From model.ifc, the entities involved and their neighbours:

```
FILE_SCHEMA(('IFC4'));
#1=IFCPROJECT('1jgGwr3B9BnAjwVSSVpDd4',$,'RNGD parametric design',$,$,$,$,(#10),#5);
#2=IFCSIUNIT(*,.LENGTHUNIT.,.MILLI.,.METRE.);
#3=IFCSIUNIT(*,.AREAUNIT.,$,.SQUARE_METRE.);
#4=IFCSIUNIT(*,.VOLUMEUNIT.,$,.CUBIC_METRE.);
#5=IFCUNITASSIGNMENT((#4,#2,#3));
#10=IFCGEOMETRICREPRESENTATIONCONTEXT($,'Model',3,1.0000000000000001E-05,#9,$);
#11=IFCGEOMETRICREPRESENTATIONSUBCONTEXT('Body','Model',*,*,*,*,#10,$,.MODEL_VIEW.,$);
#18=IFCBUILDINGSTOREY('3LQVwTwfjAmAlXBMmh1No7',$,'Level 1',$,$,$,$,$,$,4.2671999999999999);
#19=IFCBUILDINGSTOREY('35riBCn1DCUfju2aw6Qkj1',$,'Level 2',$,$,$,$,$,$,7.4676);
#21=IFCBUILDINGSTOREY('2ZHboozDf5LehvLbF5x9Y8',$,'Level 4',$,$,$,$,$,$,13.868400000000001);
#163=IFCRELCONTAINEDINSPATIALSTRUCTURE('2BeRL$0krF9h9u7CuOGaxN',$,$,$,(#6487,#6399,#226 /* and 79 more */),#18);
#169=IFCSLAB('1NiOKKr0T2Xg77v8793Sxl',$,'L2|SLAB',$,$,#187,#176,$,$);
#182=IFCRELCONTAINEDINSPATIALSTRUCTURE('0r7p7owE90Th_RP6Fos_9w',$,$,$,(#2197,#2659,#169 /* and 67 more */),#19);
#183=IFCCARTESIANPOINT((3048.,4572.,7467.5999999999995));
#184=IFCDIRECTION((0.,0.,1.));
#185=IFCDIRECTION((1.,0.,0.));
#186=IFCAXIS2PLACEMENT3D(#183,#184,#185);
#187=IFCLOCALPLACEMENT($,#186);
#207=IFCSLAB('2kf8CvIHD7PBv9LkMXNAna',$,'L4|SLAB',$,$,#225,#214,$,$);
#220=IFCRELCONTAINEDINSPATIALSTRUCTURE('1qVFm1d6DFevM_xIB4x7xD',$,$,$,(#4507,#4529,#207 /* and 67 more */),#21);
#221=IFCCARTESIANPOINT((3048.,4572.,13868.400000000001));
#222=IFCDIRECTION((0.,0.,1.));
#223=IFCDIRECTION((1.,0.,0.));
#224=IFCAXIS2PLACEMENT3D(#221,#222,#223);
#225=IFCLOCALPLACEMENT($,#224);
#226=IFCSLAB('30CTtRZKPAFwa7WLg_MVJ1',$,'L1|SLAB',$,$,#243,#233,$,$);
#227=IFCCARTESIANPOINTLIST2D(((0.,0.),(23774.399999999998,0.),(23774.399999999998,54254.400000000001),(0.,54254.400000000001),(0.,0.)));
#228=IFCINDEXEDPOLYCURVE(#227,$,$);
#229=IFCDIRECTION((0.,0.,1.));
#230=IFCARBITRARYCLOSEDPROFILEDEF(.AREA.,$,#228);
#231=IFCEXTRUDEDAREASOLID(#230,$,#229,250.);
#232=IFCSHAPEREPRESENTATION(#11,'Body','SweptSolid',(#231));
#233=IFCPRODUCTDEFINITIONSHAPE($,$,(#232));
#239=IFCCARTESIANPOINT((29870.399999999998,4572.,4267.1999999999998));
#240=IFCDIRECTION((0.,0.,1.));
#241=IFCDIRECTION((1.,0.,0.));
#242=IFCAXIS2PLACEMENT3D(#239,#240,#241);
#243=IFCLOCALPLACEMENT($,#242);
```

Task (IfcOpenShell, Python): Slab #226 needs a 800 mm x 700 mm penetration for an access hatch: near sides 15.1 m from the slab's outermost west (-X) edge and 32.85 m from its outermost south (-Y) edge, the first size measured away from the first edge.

```python
import numpy as np
import ifcopenshell
import ifcopenshell.api.feature
import ifcopenshell.api.geometry
import ifcopenshell.api.root
import ifcopenshell.geom
import ifcopenshell.util.placement
import ifcopenshell.util.representation
import ifcopenshell.util.shape
import ifcopenshell.util.unit

model = ifcopenshell.open("model.ifc")
unit_scale = ifcopenshell.util.unit.calculate_unit_scale(model)
settings = ifcopenshell.geom.settings()


def volume(element):
    """Net volume in cubic metres, openings subtracted."""
    shape = ifcopenshell.geom.create_shape(settings, element)
    return ifcopenshell.util.shape.get_volume(shape.geometry)


slab = model.by_guid("30CTtRZKPAFwa7WLg_MVJ1")
before = volume(slab)

# Extent in the slab's own axes, in metres. The edges named are its -X and -Y sides.
slab_shape = ifcopenshell.geom.create_shape(settings, slab)
vertices = ifcopenshell.util.shape.get_vertices(slab_shape.geometry)
x_min, y_min, bottom = vertices.min(axis=0)
top = vertices[:, 2].max()

opening = ifcopenshell.api.root.create_entity(model, ifc_class="IfcOpeningElement", name="Access hatch opening", predefined_type="OPENING")
context = ifcopenshell.util.representation.get_context(model, "Model", "Body", "MODEL_VIEW")
width, depth = 0.8, 0.7
outline = [(0.0, 0.0), (width, 0.0), (width, depth), (0.0, depth), (0.0, 0.0)]
# Overshoot both faces by 50 mm so the cut is clean.
shape = ifcopenshell.api.geometry.add_slab_representation(
    model, context=context, depth=top - bottom + 0.1, polyline=outline
)
ifcopenshell.api.geometry.assign_representation(model, product=opening, representation=shape)

matrix = ifcopenshell.util.placement.get_local_placement(slab.ObjectPlacement)
matrix[:, 3] = matrix @ np.append(np.array([x_min + 15.1, y_min + 32.85, bottom - 0.05]) / unit_scale, 1.0)
ifcopenshell.api.geometry.edit_object_placement(model, product=opening, matrix=matrix, is_si=False)
ifcopenshell.api.feature.add_feature(model, feature=opening, element=slab)

after = volume(slab)

print(f"slab volume {before:.3f} -> {after:.3f} m3")

model.write("model_rev.ifc")
```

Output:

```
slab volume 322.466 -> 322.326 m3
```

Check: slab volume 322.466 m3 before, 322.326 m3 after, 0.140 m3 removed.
